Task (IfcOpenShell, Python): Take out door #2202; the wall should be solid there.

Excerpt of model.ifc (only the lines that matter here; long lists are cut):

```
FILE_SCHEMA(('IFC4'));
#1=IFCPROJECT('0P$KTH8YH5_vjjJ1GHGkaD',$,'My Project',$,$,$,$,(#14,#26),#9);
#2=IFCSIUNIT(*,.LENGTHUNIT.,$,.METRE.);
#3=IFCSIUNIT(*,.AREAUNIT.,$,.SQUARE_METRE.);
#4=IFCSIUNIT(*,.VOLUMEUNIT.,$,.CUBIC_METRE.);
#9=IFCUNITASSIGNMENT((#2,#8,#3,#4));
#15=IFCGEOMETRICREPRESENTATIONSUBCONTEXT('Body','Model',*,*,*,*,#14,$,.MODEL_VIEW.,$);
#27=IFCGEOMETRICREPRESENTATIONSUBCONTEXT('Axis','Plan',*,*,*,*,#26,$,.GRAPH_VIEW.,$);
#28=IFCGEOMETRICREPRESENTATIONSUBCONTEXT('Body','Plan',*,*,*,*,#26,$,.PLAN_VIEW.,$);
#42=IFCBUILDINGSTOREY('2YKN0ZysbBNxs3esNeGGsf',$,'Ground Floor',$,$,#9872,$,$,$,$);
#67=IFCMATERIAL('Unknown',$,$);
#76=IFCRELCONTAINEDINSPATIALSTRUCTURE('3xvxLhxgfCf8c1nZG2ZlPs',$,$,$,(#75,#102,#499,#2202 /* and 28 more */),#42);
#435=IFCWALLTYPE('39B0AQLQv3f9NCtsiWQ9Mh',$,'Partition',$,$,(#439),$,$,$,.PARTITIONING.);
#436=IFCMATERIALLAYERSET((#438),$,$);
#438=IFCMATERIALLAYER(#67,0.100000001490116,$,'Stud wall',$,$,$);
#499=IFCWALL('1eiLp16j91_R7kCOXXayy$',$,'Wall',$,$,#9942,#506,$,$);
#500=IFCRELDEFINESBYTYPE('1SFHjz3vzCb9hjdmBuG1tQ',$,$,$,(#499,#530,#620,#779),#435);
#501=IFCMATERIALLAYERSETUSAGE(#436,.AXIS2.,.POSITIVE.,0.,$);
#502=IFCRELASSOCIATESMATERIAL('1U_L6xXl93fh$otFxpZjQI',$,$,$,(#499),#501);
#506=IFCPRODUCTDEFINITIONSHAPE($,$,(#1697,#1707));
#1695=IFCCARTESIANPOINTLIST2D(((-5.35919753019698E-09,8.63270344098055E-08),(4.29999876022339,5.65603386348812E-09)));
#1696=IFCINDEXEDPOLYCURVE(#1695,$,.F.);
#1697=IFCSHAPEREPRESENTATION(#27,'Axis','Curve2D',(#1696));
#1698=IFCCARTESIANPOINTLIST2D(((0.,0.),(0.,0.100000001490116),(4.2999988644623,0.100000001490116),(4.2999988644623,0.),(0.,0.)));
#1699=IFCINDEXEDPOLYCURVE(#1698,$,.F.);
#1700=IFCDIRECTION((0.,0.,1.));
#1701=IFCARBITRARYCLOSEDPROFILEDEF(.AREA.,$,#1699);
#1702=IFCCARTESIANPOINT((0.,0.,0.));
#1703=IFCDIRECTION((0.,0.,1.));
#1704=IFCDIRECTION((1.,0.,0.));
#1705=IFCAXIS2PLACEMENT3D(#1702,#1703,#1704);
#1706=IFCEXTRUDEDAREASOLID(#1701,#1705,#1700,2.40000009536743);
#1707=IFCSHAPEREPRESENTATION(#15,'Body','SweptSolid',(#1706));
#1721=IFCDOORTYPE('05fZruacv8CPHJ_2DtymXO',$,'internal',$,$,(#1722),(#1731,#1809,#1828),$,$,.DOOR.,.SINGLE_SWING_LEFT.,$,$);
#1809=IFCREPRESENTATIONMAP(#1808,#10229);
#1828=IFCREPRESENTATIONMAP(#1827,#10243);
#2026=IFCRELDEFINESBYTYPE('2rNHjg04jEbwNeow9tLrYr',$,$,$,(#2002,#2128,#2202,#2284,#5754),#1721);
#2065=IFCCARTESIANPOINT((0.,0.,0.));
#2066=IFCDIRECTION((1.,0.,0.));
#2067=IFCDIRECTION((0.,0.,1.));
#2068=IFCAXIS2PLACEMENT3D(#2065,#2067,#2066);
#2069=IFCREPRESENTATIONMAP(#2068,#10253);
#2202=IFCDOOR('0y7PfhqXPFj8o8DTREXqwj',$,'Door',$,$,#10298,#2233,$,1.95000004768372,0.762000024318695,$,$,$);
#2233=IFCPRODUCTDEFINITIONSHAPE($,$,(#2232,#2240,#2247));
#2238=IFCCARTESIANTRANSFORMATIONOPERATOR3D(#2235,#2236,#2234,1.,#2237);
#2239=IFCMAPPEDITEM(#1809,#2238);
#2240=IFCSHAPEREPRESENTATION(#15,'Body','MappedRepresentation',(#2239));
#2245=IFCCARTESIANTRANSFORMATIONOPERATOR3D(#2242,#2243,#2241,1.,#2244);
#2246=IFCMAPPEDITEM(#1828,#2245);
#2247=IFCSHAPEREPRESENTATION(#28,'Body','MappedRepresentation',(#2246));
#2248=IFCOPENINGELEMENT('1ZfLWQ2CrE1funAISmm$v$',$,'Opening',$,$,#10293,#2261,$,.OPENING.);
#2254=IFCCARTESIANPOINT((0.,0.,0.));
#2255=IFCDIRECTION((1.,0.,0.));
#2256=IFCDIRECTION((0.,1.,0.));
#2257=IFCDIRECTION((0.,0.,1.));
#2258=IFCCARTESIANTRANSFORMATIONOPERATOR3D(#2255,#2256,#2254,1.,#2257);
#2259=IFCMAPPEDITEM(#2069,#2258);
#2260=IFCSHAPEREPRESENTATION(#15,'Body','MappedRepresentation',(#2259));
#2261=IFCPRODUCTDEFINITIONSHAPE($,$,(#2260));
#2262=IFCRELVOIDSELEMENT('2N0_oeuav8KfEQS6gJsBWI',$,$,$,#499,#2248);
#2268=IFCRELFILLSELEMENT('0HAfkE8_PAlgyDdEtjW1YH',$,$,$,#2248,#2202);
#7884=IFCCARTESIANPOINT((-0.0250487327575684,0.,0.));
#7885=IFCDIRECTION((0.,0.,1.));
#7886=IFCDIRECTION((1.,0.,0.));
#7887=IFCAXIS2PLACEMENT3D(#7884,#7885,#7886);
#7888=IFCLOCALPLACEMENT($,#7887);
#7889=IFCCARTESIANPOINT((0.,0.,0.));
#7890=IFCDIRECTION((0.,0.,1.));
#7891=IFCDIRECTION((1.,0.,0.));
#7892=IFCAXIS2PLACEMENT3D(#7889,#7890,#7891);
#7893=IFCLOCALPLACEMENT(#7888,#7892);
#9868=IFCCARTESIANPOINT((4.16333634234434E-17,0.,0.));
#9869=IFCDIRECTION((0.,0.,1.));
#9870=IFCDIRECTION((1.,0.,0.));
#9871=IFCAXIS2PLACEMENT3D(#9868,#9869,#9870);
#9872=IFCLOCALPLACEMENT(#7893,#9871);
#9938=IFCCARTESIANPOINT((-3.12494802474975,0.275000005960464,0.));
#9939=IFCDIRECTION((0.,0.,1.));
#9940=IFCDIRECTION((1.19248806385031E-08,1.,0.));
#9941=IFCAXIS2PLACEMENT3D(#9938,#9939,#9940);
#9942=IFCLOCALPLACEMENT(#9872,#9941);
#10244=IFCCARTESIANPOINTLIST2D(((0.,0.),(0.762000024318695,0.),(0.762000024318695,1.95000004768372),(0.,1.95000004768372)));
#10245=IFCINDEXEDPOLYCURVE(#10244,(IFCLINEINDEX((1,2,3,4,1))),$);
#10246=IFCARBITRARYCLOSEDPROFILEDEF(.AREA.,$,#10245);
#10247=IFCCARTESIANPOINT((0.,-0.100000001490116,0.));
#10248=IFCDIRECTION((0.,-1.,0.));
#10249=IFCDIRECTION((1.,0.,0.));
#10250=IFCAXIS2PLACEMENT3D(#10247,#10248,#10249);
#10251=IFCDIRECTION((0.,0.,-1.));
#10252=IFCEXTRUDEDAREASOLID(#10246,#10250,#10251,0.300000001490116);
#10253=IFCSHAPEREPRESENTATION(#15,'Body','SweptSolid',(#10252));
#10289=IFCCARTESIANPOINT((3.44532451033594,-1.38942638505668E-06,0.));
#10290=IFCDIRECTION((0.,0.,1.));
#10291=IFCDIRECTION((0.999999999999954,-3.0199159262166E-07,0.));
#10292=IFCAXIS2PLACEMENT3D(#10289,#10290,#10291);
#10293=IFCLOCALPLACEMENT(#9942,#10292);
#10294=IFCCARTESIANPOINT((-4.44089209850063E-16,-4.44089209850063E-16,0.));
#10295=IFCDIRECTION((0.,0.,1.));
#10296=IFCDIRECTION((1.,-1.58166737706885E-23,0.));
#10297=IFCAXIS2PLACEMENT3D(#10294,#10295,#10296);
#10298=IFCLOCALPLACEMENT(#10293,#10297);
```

```python
import ifcopenshell
import ifcopenshell.api.feature
import ifcopenshell.api.root
import ifcopenshell.geom
import ifcopenshell.util.shape

model = ifcopenshell.open("model.ifc")
settings = ifcopenshell.geom.settings()


def volume(element):
    """Net volume in cubic metres, openings subtracted."""
    shape = ifcopenshell.geom.create_shape(settings, element)
    return ifcopenshell.util.shape.get_volume(shape.geometry)


door = model.by_id(2202)
opening = door.FillsVoids[0].RelatingOpeningElement
wall = opening.VoidsElements[0].RelatingBuildingElement
before = volume(wall)

ifcopenshell.api.root.remove_product(model, product=door)
ifcopenshell.api.feature.remove_feature(model, feature=opening)

after = volume(wall)

print(f"wall volume {before:.3f} -> {after:.3f} m3")

model.write("model_updated.ifc")
```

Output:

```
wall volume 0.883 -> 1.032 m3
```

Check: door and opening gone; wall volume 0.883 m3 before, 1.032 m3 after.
